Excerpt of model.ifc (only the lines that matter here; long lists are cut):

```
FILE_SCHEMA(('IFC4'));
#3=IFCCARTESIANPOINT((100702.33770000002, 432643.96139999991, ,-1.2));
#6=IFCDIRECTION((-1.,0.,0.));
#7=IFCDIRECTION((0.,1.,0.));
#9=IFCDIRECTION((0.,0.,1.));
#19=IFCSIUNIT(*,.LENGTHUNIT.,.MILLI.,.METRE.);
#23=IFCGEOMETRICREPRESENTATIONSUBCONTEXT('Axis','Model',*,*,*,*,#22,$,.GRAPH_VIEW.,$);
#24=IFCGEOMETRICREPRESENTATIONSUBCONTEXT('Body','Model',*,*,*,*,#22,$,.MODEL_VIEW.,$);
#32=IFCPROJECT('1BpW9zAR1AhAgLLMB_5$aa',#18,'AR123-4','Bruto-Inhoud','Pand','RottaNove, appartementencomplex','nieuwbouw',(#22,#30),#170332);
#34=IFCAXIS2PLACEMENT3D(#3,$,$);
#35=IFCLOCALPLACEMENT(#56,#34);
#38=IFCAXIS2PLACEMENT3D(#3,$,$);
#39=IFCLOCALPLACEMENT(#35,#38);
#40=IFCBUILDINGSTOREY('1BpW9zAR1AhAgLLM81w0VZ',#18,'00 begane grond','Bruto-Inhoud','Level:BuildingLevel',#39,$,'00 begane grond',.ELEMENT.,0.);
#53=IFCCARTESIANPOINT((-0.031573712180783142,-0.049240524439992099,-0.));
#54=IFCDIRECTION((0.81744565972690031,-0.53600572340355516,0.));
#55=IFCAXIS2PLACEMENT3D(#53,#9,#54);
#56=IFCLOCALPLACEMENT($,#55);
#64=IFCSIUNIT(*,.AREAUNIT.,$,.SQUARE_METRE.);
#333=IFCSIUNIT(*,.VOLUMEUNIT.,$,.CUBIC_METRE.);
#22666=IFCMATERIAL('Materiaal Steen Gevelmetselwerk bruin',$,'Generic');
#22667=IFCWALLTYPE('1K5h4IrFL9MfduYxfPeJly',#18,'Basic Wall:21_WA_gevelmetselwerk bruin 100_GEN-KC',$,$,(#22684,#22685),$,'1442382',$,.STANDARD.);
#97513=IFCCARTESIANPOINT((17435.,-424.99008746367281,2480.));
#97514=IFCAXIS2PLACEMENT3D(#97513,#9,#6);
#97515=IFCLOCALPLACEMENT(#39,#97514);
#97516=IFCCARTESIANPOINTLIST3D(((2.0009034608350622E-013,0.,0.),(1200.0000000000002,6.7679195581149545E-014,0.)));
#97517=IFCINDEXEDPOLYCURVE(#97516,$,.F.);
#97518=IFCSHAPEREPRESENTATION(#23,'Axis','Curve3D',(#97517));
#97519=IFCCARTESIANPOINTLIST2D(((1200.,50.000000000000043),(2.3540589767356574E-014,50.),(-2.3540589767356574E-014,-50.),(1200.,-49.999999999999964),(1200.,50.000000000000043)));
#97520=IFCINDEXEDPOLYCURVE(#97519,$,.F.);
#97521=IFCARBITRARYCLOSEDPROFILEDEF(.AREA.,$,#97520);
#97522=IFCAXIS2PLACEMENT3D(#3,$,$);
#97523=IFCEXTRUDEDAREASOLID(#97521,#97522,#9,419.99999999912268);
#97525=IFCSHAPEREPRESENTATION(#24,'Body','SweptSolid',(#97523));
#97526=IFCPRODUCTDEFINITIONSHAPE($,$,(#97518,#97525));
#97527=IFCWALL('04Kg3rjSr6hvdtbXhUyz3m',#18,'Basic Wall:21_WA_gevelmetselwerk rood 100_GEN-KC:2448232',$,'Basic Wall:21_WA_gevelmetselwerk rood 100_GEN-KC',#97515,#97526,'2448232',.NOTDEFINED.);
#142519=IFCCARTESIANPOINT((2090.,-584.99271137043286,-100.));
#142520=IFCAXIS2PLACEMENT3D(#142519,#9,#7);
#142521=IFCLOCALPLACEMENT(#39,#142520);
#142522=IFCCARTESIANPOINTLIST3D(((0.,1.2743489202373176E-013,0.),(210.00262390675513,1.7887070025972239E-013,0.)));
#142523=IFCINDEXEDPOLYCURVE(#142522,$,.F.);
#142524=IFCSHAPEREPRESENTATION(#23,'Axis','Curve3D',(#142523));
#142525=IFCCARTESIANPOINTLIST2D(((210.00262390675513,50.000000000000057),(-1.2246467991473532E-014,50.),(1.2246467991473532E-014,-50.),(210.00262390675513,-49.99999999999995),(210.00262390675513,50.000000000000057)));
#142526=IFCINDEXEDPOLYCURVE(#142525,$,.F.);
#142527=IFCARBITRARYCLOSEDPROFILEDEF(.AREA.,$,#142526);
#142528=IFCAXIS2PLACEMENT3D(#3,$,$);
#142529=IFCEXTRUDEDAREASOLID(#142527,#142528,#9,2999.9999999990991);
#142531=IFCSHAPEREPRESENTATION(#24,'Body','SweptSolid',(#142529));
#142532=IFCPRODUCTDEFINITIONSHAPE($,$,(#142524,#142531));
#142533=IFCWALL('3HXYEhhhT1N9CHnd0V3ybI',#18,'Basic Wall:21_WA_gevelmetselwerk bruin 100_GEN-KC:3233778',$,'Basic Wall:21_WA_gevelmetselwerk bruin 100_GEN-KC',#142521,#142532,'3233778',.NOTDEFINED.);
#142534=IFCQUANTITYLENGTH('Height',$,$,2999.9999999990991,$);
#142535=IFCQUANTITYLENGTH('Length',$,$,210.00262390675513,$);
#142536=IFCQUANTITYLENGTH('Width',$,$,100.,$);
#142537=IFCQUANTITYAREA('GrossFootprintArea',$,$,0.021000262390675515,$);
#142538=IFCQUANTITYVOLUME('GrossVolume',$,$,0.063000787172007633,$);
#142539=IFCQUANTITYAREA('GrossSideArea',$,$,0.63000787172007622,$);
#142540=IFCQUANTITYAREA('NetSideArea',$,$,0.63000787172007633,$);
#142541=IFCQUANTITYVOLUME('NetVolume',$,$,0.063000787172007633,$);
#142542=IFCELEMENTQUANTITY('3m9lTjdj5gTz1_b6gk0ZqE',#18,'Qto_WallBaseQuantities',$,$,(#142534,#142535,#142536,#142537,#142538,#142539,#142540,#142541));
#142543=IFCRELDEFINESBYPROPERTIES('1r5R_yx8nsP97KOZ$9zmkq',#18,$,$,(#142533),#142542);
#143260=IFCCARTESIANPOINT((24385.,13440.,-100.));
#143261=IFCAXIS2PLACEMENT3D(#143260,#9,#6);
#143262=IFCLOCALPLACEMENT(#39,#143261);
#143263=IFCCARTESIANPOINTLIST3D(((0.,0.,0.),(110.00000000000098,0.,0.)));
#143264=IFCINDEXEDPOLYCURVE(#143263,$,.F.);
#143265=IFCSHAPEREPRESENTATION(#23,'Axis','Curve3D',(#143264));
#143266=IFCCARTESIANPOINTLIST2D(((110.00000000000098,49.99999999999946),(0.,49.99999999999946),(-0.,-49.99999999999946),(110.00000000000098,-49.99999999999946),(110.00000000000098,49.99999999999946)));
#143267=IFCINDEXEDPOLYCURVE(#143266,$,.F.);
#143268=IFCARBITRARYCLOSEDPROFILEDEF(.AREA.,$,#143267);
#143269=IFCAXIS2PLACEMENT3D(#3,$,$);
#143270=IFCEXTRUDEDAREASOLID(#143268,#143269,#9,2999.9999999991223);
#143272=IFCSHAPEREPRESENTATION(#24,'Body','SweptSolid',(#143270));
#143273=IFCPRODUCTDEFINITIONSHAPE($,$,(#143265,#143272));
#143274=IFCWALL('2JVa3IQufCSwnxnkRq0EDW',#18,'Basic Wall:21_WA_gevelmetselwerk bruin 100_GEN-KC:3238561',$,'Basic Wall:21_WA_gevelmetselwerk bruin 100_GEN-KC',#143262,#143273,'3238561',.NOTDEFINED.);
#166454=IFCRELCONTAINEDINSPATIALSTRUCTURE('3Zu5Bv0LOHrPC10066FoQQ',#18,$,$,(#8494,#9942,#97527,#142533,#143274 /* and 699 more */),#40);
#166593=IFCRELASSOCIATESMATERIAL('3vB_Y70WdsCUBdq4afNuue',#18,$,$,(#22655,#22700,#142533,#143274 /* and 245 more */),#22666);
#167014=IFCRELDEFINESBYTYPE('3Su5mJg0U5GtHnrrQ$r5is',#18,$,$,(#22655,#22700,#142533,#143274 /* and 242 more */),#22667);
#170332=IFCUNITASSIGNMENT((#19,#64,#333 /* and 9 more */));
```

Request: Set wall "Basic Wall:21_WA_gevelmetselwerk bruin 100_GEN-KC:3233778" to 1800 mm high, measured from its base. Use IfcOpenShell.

```python
import ifcopenshell
import ifcopenshell.api.pset
import ifcopenshell.geom
import ifcopenshell.util.element
import ifcopenshell.util.representation
import ifcopenshell.util.shape
import ifcopenshell.util.unit

model = ifcopenshell.open("model.ifc")
unit_scale = ifcopenshell.util.unit.calculate_unit_scale(model)
area_scale = ifcopenshell.util.unit.calculate_unit_scale(model, "AREAUNIT")
volume_scale = ifcopenshell.util.unit.calculate_unit_scale(model, "VOLUMEUNIT")
settings = ifcopenshell.geom.settings()


def volume(element):
    """Net volume in cubic metres, openings subtracted."""
    shape = ifcopenshell.geom.create_shape(settings, element)
    return ifcopenshell.util.shape.get_volume(shape.geometry)


wall = model.by_id(142533)
before = volume(wall)

body = ifcopenshell.util.representation.get_representation(wall, "Model", "Body")
solid = body.Items[0]
old_height = solid.Depth
solid.Depth = 1.8 / unit_scale
after = volume(wall)
thickness = 0.1  # wall thickness in metres

# Update the stored height, areas and volumes.
qto = model.by_id(ifcopenshell.util.element.get_pset(wall, "Qto_WallBaseQuantities", should_inherit=False)["id"])
ifcopenshell.api.pset.edit_qto(model, qto=qto, properties={
    "Height": solid.Depth,
    "GrossVolume": ifcopenshell.util.element.get_pset(wall, "Qto_WallBaseQuantities", "GrossVolume") * solid.Depth / old_height,
    "GrossSideArea": ifcopenshell.util.element.get_pset(wall, "Qto_WallBaseQuantities", "GrossSideArea") * solid.Depth / old_height,
    "NetSideArea": after / thickness / area_scale,
    "NetVolume": after / volume_scale,
})

print(f"height {old_height:g} -> {solid.Depth:g}, volume {before:.3f} -> {after:.3f} m3")

model.write("model-out.ifc")
```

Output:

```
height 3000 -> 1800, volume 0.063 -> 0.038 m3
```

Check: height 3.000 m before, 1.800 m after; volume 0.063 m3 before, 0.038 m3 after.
